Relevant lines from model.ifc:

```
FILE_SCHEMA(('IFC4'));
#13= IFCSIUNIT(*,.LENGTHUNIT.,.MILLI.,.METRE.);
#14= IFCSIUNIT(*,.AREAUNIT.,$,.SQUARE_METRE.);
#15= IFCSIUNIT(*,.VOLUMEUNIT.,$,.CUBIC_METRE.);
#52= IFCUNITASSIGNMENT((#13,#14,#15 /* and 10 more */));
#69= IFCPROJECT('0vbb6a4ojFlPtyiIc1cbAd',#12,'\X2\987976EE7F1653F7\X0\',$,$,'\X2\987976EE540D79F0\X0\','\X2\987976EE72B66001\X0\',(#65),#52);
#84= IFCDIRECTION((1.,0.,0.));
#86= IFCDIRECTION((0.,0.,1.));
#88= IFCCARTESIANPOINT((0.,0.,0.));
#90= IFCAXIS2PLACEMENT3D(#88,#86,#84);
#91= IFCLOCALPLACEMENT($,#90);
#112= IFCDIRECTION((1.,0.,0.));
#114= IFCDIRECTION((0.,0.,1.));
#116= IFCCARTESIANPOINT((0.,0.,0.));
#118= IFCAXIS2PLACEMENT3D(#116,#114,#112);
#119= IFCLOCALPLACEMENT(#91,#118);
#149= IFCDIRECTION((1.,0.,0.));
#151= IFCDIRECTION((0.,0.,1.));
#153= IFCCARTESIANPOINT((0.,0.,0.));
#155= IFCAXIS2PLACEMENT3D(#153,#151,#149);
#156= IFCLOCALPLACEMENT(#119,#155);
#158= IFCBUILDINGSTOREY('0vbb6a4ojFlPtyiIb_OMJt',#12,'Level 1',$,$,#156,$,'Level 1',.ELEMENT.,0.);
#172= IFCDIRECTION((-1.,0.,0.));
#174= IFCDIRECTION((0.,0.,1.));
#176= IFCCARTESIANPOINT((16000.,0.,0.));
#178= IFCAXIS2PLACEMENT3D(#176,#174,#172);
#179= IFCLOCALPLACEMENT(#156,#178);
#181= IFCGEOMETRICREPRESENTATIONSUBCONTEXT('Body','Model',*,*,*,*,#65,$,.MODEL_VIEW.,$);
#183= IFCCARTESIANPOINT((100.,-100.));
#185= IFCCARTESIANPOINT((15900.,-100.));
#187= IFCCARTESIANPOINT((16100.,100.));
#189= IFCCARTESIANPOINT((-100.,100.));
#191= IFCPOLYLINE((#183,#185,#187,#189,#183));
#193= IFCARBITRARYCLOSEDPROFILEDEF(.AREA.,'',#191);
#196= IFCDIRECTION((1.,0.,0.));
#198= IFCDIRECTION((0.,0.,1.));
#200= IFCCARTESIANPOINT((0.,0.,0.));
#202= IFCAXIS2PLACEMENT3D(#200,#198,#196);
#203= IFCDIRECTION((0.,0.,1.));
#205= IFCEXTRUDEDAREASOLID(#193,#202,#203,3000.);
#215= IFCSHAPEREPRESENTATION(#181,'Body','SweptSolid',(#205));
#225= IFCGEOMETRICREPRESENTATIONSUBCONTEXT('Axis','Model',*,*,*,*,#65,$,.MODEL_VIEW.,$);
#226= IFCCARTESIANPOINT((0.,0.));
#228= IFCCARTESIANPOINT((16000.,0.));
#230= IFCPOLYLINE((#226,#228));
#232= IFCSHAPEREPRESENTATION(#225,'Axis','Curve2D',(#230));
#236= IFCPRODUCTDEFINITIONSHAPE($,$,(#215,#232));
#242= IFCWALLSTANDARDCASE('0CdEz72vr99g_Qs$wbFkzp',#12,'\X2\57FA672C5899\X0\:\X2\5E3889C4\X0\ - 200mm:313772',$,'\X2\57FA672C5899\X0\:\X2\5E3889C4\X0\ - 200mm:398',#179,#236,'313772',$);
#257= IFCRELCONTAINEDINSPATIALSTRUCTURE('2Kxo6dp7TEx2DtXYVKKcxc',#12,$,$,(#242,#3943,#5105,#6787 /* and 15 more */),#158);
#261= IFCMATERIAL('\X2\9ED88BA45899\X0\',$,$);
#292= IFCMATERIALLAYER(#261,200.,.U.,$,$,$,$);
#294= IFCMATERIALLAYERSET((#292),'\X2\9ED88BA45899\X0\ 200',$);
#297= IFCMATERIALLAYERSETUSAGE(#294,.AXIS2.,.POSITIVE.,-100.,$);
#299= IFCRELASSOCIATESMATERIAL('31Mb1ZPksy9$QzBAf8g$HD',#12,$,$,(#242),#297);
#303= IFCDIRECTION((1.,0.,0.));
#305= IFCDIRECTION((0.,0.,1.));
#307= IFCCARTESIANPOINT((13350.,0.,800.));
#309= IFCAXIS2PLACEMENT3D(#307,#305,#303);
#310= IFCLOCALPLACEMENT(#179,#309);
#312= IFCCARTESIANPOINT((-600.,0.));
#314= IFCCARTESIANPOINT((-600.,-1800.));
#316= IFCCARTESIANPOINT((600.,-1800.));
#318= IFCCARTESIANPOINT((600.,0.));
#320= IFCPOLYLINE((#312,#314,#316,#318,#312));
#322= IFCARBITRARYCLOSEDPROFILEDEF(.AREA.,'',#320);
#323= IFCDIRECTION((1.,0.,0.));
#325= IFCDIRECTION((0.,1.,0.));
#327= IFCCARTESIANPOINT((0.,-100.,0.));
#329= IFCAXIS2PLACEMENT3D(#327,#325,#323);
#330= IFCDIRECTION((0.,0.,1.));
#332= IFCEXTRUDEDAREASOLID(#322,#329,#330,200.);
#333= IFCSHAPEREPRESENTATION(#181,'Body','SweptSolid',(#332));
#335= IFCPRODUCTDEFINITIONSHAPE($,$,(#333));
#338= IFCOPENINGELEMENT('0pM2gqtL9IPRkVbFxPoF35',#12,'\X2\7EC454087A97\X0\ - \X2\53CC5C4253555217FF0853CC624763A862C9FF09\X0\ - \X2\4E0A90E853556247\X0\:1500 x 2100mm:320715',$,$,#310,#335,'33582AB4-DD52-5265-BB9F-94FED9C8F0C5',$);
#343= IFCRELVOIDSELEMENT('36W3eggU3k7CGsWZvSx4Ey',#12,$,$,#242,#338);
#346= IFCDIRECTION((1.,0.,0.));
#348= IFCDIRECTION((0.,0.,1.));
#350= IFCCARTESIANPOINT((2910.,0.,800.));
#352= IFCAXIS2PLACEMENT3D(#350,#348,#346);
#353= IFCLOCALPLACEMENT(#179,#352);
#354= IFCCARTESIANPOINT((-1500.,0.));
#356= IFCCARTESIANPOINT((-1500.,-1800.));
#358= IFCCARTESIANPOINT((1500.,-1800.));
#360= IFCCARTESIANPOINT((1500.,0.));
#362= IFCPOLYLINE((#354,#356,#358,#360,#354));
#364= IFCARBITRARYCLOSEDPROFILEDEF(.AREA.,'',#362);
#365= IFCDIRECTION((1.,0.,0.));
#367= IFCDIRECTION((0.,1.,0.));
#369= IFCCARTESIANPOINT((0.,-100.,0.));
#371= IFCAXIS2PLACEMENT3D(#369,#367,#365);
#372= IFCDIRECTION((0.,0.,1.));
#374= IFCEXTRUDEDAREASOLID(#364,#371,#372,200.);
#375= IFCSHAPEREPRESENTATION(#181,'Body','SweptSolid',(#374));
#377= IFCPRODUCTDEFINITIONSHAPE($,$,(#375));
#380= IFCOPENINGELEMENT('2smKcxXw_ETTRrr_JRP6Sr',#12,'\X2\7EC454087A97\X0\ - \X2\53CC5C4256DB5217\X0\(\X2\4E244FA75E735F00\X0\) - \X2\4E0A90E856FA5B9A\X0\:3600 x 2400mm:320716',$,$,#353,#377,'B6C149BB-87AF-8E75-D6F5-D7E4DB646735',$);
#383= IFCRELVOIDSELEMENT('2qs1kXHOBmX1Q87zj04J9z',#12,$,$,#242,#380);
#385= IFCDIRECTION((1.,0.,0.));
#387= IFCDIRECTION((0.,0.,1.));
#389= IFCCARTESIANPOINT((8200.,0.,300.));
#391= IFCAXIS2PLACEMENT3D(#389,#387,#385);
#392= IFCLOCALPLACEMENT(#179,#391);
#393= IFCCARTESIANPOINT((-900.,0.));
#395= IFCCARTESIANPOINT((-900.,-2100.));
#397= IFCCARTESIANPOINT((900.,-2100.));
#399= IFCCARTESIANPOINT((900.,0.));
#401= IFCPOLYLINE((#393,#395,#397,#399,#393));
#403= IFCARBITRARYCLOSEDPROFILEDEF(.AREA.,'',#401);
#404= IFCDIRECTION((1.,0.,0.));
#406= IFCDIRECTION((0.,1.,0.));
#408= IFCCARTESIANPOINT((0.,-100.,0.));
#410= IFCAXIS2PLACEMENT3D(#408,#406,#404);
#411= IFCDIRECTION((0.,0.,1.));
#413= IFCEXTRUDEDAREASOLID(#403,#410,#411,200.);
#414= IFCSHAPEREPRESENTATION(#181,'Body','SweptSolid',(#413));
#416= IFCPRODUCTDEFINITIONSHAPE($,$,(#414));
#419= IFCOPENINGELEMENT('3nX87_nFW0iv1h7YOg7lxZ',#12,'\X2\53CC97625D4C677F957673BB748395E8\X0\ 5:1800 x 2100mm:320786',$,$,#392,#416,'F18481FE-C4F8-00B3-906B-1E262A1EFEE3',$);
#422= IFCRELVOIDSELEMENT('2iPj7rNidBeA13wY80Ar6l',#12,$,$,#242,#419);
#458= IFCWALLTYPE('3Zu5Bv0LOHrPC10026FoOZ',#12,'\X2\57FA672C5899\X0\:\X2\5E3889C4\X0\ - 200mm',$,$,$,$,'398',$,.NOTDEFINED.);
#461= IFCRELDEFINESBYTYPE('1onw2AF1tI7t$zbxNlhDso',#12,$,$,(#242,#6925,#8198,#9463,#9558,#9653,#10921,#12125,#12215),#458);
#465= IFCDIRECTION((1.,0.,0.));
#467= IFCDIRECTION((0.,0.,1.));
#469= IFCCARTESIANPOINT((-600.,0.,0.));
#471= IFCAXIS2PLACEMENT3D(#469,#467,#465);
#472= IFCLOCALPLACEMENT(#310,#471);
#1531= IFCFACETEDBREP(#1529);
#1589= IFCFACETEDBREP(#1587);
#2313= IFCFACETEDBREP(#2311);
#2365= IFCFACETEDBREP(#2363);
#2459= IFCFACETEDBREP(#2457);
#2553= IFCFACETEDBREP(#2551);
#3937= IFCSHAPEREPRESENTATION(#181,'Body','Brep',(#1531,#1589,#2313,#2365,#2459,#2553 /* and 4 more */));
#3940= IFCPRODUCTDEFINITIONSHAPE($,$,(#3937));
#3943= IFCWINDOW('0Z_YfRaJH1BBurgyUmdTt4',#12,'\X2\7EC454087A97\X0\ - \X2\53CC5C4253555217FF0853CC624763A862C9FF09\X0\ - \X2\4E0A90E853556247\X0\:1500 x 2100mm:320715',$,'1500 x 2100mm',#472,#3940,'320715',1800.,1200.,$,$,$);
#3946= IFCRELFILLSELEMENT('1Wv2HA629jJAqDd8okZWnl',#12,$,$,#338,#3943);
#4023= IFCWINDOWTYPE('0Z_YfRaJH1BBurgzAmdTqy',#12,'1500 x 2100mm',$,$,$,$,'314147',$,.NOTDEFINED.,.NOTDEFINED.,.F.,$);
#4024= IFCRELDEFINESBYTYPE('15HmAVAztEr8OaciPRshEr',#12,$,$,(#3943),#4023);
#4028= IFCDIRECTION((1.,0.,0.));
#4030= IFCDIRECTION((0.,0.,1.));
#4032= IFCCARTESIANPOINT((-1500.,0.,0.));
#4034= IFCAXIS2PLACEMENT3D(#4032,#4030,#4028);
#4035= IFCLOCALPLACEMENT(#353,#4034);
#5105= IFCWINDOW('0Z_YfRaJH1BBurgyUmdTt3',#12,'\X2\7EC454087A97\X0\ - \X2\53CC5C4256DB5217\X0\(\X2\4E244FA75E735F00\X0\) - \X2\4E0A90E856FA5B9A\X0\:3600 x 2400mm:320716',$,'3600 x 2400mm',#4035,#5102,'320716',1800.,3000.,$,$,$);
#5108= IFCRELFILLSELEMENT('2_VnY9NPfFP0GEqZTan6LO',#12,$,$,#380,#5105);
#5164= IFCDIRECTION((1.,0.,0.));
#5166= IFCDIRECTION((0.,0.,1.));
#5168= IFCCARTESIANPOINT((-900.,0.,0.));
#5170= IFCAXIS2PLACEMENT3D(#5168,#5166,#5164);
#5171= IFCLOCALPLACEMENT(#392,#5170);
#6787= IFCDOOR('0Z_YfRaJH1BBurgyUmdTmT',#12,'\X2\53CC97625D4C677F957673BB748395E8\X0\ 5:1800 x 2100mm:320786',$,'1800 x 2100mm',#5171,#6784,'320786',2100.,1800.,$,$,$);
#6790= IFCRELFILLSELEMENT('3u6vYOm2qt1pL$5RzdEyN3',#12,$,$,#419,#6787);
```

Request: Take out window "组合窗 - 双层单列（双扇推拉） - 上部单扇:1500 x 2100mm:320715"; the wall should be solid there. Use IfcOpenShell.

```python
import ifcopenshell
import ifcopenshell.api.feature
import ifcopenshell.api.root
import ifcopenshell.geom
import ifcopenshell.util.shape

model = ifcopenshell.open("model.ifc")
settings = ifcopenshell.geom.settings()


def volume(element):
    """Net volume in cubic metres, openings subtracted."""
    shape = ifcopenshell.geom.create_shape(settings, element)
    return ifcopenshell.util.shape.get_volume(shape.geometry)


window = model.by_guid("0Z_YfRaJH1BBurgyUmdTt4")
opening = window.FillsVoids[0].RelatingOpeningElement
wall = opening.VoidsElements[0].RelatingBuildingElement
before = volume(wall)

ifcopenshell.api.root.remove_product(model, product=window)
ifcopenshell.api.feature.remove_feature(model, feature=opening)

after = volume(wall)

print(f"wall volume {before:.3f} -> {after:.3f} m3")

model.write("model_updated.ifc")
```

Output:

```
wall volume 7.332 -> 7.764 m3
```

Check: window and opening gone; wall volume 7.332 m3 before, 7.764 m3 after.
